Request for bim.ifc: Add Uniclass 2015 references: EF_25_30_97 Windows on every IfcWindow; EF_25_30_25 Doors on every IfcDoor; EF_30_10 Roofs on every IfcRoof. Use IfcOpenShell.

First a look at what the model holds.

```python
import ifcopenshell

model = ifcopenshell.open("bim.ifc")
print(model.schema)
print("classifications:", [c.Name for c in model.by_type("IfcClassification")])
for ifc_class in ("IfcDoor", "IfcRoof", "IfcStair", "IfcWall", "IfcWindow"):
    print(ifc_class, len(model.by_type(ifc_class)))
```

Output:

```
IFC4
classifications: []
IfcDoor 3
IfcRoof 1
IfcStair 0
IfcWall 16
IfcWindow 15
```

```python
import ifcopenshell
import ifcopenshell.api.classification

model = ifcopenshell.open("bim.ifc")

system = ifcopenshell.api.classification.add_classification(model, classification="Uniclass 2015")

codes = {
    "IfcWindow": ("EF_25_30_97", "Windows"),
    "IfcDoor": ("EF_25_30_25", "Doors"),
    "IfcRoof": ("EF_30_10", "Roofs"),
}
for ifc_class, (code, name) in codes.items():
    products = model.by_type(ifc_class)
    ifcopenshell.api.classification.add_reference(
        model, products=products, classification=system, identification=code, name=name
    )
    print(code, len(products))

model.write("bim_edited.ifc")
```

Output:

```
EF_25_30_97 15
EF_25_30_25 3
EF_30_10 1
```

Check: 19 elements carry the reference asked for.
